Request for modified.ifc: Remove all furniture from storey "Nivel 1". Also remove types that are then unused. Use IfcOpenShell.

First a look at what the model holds.

```python
import ifcopenshell
import ifcopenshell.util.element

model = ifcopenshell.open("modified.ifc")
print(model.schema)
storey = next(s for s in model.by_type("IfcBuildingStorey") if s.Name == "Nivel 1")
furniture = [e for e in ifcopenshell.util.element.get_decomposition(storey) if e.is_a("IfcFurnishingElement")]
seen = {}
for e in furniture:
    element_type = ifcopenshell.util.element.get_type(e)
    name = element_type.Name if element_type not in (None, e) else None
    seen[name] = seen.get(name, 0) + 1
for name, count in sorted(seen.items(), key=str):
    print(count, "x", name)
```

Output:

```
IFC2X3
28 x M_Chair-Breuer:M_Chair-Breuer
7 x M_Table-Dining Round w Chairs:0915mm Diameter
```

```python
import ifcopenshell
import ifcopenshell.api.root
import ifcopenshell.util.element

model = ifcopenshell.open("modified.ifc")

storey = next(s for s in model.by_type("IfcBuildingStorey") if s.Name == "Nivel 1")
furniture = [e for e in ifcopenshell.util.element.get_decomposition(storey) if e.is_a("IfcFurnishingElement")]
types = {ifcopenshell.util.element.get_type(e) for e in furniture} - {None, *furniture}

for e in furniture:
    ifcopenshell.api.root.remove_product(model, product=e)
print(len(furniture), "removed")

unused = [t for t in types if not ifcopenshell.util.element.get_types(t)]
for t in unused:
    ifcopenshell.api.root.remove_product(model, product=t)
print(len(unused), "unused types removed")

model.write("modified-out.ifc")
```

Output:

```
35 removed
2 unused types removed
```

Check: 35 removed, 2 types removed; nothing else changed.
